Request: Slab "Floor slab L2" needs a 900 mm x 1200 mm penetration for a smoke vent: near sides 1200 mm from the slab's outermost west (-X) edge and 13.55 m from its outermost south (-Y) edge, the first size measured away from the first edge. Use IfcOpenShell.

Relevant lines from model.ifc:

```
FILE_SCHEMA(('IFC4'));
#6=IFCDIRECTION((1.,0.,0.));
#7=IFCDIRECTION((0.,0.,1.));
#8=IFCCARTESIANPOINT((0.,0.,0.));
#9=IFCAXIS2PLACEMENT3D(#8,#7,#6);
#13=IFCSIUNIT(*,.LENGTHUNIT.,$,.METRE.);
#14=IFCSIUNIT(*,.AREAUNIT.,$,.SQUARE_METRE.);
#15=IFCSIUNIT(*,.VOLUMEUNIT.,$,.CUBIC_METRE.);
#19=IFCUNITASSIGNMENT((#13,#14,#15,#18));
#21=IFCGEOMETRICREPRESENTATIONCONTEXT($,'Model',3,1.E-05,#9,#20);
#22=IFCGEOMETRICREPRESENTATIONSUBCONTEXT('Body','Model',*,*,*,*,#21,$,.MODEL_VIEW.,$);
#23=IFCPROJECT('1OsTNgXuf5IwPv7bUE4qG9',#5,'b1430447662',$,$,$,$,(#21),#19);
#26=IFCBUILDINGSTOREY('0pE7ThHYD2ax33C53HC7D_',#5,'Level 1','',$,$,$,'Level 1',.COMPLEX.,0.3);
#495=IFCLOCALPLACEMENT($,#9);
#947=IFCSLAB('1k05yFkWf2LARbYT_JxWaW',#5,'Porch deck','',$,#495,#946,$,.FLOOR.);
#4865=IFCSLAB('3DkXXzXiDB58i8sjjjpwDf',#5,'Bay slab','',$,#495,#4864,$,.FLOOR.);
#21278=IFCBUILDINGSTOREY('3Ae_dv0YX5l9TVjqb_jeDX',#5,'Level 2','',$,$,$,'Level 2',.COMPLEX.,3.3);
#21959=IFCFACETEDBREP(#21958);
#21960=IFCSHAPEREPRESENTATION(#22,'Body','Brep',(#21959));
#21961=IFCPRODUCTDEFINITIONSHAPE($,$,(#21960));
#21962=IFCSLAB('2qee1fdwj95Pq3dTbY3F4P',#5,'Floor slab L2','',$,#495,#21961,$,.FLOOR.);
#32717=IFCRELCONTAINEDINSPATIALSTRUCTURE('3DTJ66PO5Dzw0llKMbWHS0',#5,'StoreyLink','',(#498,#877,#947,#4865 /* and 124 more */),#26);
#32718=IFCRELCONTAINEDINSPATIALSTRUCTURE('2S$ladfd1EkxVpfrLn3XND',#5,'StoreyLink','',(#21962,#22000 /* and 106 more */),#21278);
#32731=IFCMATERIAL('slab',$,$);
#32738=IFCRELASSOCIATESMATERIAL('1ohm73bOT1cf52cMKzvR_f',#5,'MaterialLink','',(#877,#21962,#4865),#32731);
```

```python
import numpy as np
import ifcopenshell
import ifcopenshell.api.feature
import ifcopenshell.api.geometry
import ifcopenshell.api.root
import ifcopenshell.geom
import ifcopenshell.util.placement
import ifcopenshell.util.representation
import ifcopenshell.util.shape
import ifcopenshell.util.unit

model = ifcopenshell.open("model.ifc")
unit_scale = ifcopenshell.util.unit.calculate_unit_scale(model)
settings = ifcopenshell.geom.settings()


def volume(element):
    """Net volume in cubic metres, openings subtracted."""
    shape = ifcopenshell.geom.create_shape(settings, element)
    return ifcopenshell.util.shape.get_volume(shape.geometry)


slab = model.by_guid("2qee1fdwj95Pq3dTbY3F4P")
before = volume(slab)

# Extent in the slab's own axes, in metres. The edges named are its -X and -Y sides.
slab_shape = ifcopenshell.geom.create_shape(settings, slab)
vertices = ifcopenshell.util.shape.get_vertices(slab_shape.geometry)
x_min, y_min, bottom = vertices.min(axis=0)
top = vertices[:, 2].max()

opening = ifcopenshell.api.root.create_entity(model, ifc_class="IfcOpeningElement", name="Smoke vent opening", predefined_type="OPENING")
context = ifcopenshell.util.representation.get_context(model, "Model", "Body", "MODEL_VIEW")
width, depth = 0.9, 1.2
outline = [(0.0, 0.0), (width, 0.0), (width, depth), (0.0, depth), (0.0, 0.0)]
# Overshoot both faces by 50 mm so the cut is clean.
shape = ifcopenshell.api.geometry.add_slab_representation(
    model, context=context, depth=top - bottom + 0.1, polyline=outline
)
ifcopenshell.api.geometry.assign_representation(model, product=opening, representation=shape)

matrix = ifcopenshell.util.placement.get_local_placement(slab.ObjectPlacement)
matrix[:, 3] = matrix @ np.append(np.array([x_min + 1.2, y_min + 13.55, bottom - 0.05]) / unit_scale, 1.0)
ifcopenshell.api.geometry.edit_object_placement(model, product=opening, matrix=matrix, is_si=False)
ifcopenshell.api.feature.add_feature(model, feature=opening, element=slab)

after = volume(slab)

print(f"slab volume {before:.3f} -> {after:.3f} m3")

model.write("model_rev.ifc")
```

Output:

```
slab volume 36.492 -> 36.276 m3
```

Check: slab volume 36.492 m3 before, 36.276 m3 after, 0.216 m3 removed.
